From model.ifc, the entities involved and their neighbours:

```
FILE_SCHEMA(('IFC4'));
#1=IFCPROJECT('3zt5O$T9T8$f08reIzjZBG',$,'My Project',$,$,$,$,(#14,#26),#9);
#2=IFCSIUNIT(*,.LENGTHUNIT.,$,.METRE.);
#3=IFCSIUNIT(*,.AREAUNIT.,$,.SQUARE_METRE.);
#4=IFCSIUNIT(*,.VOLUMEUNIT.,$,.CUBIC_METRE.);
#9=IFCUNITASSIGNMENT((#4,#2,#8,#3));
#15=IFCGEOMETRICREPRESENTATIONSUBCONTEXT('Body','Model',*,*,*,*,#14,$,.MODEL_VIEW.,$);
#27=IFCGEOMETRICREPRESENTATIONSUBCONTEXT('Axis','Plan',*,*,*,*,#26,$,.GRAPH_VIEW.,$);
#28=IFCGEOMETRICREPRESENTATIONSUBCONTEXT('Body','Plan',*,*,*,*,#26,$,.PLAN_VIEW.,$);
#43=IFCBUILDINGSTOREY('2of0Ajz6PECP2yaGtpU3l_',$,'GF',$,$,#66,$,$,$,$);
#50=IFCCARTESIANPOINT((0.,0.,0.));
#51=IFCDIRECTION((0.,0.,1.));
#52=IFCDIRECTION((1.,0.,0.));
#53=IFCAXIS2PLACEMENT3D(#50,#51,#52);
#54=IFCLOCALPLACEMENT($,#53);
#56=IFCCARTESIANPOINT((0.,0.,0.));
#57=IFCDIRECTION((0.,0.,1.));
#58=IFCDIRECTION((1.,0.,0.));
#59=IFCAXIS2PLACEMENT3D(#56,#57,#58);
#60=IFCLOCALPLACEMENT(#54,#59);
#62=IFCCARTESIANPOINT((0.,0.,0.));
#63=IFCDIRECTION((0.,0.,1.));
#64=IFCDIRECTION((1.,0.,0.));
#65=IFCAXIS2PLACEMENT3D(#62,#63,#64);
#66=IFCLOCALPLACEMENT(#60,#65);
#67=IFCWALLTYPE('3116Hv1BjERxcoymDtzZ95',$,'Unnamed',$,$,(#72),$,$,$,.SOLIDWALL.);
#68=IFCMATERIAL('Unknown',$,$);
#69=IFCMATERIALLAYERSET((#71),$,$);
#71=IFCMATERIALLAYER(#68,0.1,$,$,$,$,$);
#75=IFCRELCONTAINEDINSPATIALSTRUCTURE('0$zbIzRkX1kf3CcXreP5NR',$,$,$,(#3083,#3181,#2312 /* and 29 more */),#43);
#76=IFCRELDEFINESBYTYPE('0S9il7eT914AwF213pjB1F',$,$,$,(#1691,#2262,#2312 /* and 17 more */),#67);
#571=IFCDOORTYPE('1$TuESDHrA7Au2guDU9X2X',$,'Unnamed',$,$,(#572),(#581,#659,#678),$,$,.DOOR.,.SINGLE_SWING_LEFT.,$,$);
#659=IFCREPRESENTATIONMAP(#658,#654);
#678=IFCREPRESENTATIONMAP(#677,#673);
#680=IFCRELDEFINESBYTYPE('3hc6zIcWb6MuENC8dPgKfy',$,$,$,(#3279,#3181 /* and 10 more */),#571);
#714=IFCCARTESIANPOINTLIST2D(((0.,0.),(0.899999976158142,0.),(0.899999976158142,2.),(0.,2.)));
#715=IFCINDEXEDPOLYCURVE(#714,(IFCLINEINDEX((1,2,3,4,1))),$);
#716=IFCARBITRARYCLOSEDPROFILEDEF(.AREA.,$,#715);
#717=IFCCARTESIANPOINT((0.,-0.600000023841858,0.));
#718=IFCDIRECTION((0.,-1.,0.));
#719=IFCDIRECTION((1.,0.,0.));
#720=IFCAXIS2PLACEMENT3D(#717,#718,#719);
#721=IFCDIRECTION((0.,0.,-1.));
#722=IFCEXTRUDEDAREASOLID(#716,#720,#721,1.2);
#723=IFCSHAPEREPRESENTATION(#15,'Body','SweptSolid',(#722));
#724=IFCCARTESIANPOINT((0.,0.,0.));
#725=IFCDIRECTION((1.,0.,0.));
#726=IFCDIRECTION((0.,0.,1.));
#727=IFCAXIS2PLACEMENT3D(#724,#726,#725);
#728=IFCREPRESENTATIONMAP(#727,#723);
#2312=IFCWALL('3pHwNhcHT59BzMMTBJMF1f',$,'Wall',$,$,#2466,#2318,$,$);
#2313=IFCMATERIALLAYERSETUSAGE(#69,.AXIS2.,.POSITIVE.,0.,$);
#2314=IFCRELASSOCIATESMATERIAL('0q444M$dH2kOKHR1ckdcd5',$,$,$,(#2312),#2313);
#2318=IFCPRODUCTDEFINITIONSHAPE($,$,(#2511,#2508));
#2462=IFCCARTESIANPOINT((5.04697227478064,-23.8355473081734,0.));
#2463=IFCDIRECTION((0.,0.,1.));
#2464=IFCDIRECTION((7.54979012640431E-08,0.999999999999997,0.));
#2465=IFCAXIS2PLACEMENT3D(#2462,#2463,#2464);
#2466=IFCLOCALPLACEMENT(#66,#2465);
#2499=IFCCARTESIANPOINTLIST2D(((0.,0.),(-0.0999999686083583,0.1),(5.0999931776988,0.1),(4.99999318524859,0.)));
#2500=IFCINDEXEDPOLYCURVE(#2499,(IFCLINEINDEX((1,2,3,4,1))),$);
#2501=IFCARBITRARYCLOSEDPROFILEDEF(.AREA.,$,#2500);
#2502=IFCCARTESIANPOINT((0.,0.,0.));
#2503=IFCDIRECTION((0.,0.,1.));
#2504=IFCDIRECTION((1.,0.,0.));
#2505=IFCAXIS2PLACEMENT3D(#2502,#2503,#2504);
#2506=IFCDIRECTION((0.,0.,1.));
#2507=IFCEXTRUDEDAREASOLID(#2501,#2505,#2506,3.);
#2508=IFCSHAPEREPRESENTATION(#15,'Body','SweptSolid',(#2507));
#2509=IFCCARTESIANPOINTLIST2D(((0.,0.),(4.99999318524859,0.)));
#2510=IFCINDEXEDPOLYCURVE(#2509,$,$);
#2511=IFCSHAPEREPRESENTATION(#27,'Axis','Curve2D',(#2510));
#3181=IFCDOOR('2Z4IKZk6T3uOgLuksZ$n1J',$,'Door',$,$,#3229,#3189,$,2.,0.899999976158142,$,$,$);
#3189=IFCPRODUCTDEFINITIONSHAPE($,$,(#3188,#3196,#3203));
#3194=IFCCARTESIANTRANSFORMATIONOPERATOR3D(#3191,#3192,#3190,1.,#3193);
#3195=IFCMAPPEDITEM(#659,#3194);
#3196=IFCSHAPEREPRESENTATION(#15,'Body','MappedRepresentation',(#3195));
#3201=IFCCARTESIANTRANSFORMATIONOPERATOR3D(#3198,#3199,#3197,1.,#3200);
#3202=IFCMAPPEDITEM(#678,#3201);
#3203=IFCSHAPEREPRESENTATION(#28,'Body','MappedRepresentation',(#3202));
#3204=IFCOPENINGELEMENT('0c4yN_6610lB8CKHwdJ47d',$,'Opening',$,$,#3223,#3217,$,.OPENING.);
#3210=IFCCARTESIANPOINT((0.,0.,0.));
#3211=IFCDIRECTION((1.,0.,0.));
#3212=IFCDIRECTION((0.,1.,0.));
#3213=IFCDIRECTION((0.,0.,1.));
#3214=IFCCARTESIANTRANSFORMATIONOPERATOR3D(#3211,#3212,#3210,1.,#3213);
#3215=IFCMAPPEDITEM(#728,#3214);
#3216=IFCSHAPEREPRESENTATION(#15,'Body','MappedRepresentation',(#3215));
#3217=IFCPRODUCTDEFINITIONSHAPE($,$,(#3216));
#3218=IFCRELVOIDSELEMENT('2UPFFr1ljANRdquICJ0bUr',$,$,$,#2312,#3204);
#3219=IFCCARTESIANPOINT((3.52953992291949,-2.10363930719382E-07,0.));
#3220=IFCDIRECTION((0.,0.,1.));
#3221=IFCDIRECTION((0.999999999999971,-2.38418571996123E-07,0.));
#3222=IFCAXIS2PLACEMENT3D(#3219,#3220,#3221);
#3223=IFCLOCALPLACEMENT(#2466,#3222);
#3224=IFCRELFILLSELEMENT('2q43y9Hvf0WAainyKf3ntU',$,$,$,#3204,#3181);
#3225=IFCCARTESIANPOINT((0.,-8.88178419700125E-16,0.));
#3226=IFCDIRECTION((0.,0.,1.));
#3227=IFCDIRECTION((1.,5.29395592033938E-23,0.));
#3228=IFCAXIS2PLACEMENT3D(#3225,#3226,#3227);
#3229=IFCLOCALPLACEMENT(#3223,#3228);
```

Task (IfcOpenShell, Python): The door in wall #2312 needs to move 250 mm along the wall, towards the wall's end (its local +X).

```python
import ifcopenshell
import ifcopenshell.api.geometry
import ifcopenshell.util.placement
import ifcopenshell.util.unit

model = ifcopenshell.open("model.ifc")
unit_scale = ifcopenshell.util.unit.calculate_unit_scale(model)

door = model.by_id(3181)
opening = door.FillsVoids[0].RelatingOpeningElement
wall = opening.VoidsElements[0].RelatingBuildingElement

wall_matrix = ifcopenshell.util.placement.get_local_placement(wall.ObjectPlacement)
shift = wall_matrix[:3, 0] * 0.25 / unit_scale
before = ifcopenshell.util.placement.get_local_placement(door.ObjectPlacement)[:3, 3].copy()

# The door is placed relative to its opening, so it follows when the opening moves.
matrix = ifcopenshell.util.placement.get_local_placement(opening.ObjectPlacement)
matrix[:3, 3] += shift
ifcopenshell.api.geometry.edit_object_placement(
    model, product=opening, matrix=matrix, is_si=False, should_transform_children=True
)

after = ifcopenshell.util.placement.get_local_placement(door.ObjectPlacement)[:3, 3]
print("door moved by", (after - before).round(3) + 0.0)

model.write("model_rev.ifc")
```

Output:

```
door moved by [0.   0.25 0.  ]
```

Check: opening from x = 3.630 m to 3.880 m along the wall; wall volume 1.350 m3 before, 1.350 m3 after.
